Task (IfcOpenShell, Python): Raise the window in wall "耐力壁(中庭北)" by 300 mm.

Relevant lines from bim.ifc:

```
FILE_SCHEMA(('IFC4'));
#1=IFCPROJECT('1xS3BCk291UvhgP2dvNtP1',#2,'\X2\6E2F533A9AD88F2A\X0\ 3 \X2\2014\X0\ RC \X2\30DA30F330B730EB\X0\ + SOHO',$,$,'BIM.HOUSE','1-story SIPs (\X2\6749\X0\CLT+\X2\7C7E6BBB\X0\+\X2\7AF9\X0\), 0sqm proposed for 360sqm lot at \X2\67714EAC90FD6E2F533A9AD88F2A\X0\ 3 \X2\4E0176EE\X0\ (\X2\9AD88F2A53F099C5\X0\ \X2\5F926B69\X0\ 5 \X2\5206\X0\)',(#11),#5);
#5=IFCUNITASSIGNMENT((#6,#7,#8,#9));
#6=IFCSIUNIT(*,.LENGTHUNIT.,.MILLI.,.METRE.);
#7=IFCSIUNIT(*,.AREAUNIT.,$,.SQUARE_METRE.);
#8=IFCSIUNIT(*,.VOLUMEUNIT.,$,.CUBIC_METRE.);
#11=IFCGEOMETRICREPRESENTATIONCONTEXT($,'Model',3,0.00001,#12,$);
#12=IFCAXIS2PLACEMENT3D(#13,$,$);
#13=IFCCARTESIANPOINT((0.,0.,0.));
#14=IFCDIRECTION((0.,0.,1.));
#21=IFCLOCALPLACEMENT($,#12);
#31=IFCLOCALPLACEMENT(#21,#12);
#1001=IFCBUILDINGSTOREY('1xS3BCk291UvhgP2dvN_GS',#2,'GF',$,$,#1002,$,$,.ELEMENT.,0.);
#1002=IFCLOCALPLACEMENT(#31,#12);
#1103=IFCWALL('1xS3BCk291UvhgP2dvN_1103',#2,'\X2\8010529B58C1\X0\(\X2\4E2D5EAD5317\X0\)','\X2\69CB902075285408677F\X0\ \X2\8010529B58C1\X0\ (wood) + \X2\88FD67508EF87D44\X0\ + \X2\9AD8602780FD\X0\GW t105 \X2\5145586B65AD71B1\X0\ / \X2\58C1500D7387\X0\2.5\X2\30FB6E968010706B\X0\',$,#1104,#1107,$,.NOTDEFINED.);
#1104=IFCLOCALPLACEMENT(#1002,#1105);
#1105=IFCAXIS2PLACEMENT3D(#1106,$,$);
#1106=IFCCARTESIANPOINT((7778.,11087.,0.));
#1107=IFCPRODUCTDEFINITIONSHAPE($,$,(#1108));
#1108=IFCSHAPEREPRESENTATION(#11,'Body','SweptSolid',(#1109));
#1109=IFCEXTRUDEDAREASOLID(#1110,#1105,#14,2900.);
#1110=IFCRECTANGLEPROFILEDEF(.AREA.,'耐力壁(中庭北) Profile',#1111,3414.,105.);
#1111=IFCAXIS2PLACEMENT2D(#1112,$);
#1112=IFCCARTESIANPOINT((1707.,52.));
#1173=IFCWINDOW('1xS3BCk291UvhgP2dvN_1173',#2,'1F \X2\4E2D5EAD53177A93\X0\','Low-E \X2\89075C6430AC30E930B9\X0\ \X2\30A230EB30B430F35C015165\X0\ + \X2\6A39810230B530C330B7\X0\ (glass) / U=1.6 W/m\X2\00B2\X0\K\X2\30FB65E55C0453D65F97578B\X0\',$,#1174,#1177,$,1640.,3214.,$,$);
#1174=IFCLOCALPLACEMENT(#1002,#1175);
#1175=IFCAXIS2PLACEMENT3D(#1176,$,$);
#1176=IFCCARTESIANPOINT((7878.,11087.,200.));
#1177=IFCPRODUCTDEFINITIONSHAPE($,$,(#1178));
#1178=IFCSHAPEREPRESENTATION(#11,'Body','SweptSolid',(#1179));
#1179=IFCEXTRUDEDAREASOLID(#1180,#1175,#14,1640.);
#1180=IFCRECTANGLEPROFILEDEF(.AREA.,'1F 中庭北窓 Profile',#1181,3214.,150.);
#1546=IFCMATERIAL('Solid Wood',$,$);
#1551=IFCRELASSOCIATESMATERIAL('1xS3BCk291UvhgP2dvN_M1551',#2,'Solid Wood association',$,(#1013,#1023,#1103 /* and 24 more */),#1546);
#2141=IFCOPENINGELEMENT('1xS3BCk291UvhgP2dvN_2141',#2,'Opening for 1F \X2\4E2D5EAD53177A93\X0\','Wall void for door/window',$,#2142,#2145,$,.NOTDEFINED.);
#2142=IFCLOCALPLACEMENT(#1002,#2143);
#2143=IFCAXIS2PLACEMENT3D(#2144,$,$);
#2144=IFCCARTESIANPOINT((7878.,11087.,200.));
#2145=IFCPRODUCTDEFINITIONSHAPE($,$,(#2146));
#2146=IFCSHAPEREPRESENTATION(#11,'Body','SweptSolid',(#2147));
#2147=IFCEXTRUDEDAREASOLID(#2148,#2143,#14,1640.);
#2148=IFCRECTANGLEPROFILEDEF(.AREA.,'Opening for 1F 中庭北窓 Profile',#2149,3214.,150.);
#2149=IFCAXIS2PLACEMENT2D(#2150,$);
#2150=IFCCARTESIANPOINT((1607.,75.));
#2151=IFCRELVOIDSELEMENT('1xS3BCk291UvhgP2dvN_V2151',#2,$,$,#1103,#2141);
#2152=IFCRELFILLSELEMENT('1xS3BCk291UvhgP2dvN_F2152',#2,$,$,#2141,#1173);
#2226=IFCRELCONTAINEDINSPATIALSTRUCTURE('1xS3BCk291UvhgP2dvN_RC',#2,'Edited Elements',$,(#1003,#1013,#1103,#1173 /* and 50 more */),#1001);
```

```python
import numpy as np
import ifcopenshell
import ifcopenshell.api.geometry
import ifcopenshell.util.placement
import ifcopenshell.util.unit

model = ifcopenshell.open("bim.ifc")
unit_scale = ifcopenshell.util.unit.calculate_unit_scale(model)

window = model.by_id(1173)
opening = window.FillsVoids[0].RelatingOpeningElement
dz = 300.0

shift = np.array([0.0, 0.0, dz])
# The window is not placed relative to its opening, so move both.
for product in (opening, window):
    matrix = ifcopenshell.util.placement.get_local_placement(product.ObjectPlacement)
    matrix[:3, 3] += shift
    ifcopenshell.api.geometry.edit_object_placement(model, product=product, matrix=matrix, is_si=False)

print(f"moved by {dz * unit_scale:+.3f} m")

model.write("bim_edited.ifc")
```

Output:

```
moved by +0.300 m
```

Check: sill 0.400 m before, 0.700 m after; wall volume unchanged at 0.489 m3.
